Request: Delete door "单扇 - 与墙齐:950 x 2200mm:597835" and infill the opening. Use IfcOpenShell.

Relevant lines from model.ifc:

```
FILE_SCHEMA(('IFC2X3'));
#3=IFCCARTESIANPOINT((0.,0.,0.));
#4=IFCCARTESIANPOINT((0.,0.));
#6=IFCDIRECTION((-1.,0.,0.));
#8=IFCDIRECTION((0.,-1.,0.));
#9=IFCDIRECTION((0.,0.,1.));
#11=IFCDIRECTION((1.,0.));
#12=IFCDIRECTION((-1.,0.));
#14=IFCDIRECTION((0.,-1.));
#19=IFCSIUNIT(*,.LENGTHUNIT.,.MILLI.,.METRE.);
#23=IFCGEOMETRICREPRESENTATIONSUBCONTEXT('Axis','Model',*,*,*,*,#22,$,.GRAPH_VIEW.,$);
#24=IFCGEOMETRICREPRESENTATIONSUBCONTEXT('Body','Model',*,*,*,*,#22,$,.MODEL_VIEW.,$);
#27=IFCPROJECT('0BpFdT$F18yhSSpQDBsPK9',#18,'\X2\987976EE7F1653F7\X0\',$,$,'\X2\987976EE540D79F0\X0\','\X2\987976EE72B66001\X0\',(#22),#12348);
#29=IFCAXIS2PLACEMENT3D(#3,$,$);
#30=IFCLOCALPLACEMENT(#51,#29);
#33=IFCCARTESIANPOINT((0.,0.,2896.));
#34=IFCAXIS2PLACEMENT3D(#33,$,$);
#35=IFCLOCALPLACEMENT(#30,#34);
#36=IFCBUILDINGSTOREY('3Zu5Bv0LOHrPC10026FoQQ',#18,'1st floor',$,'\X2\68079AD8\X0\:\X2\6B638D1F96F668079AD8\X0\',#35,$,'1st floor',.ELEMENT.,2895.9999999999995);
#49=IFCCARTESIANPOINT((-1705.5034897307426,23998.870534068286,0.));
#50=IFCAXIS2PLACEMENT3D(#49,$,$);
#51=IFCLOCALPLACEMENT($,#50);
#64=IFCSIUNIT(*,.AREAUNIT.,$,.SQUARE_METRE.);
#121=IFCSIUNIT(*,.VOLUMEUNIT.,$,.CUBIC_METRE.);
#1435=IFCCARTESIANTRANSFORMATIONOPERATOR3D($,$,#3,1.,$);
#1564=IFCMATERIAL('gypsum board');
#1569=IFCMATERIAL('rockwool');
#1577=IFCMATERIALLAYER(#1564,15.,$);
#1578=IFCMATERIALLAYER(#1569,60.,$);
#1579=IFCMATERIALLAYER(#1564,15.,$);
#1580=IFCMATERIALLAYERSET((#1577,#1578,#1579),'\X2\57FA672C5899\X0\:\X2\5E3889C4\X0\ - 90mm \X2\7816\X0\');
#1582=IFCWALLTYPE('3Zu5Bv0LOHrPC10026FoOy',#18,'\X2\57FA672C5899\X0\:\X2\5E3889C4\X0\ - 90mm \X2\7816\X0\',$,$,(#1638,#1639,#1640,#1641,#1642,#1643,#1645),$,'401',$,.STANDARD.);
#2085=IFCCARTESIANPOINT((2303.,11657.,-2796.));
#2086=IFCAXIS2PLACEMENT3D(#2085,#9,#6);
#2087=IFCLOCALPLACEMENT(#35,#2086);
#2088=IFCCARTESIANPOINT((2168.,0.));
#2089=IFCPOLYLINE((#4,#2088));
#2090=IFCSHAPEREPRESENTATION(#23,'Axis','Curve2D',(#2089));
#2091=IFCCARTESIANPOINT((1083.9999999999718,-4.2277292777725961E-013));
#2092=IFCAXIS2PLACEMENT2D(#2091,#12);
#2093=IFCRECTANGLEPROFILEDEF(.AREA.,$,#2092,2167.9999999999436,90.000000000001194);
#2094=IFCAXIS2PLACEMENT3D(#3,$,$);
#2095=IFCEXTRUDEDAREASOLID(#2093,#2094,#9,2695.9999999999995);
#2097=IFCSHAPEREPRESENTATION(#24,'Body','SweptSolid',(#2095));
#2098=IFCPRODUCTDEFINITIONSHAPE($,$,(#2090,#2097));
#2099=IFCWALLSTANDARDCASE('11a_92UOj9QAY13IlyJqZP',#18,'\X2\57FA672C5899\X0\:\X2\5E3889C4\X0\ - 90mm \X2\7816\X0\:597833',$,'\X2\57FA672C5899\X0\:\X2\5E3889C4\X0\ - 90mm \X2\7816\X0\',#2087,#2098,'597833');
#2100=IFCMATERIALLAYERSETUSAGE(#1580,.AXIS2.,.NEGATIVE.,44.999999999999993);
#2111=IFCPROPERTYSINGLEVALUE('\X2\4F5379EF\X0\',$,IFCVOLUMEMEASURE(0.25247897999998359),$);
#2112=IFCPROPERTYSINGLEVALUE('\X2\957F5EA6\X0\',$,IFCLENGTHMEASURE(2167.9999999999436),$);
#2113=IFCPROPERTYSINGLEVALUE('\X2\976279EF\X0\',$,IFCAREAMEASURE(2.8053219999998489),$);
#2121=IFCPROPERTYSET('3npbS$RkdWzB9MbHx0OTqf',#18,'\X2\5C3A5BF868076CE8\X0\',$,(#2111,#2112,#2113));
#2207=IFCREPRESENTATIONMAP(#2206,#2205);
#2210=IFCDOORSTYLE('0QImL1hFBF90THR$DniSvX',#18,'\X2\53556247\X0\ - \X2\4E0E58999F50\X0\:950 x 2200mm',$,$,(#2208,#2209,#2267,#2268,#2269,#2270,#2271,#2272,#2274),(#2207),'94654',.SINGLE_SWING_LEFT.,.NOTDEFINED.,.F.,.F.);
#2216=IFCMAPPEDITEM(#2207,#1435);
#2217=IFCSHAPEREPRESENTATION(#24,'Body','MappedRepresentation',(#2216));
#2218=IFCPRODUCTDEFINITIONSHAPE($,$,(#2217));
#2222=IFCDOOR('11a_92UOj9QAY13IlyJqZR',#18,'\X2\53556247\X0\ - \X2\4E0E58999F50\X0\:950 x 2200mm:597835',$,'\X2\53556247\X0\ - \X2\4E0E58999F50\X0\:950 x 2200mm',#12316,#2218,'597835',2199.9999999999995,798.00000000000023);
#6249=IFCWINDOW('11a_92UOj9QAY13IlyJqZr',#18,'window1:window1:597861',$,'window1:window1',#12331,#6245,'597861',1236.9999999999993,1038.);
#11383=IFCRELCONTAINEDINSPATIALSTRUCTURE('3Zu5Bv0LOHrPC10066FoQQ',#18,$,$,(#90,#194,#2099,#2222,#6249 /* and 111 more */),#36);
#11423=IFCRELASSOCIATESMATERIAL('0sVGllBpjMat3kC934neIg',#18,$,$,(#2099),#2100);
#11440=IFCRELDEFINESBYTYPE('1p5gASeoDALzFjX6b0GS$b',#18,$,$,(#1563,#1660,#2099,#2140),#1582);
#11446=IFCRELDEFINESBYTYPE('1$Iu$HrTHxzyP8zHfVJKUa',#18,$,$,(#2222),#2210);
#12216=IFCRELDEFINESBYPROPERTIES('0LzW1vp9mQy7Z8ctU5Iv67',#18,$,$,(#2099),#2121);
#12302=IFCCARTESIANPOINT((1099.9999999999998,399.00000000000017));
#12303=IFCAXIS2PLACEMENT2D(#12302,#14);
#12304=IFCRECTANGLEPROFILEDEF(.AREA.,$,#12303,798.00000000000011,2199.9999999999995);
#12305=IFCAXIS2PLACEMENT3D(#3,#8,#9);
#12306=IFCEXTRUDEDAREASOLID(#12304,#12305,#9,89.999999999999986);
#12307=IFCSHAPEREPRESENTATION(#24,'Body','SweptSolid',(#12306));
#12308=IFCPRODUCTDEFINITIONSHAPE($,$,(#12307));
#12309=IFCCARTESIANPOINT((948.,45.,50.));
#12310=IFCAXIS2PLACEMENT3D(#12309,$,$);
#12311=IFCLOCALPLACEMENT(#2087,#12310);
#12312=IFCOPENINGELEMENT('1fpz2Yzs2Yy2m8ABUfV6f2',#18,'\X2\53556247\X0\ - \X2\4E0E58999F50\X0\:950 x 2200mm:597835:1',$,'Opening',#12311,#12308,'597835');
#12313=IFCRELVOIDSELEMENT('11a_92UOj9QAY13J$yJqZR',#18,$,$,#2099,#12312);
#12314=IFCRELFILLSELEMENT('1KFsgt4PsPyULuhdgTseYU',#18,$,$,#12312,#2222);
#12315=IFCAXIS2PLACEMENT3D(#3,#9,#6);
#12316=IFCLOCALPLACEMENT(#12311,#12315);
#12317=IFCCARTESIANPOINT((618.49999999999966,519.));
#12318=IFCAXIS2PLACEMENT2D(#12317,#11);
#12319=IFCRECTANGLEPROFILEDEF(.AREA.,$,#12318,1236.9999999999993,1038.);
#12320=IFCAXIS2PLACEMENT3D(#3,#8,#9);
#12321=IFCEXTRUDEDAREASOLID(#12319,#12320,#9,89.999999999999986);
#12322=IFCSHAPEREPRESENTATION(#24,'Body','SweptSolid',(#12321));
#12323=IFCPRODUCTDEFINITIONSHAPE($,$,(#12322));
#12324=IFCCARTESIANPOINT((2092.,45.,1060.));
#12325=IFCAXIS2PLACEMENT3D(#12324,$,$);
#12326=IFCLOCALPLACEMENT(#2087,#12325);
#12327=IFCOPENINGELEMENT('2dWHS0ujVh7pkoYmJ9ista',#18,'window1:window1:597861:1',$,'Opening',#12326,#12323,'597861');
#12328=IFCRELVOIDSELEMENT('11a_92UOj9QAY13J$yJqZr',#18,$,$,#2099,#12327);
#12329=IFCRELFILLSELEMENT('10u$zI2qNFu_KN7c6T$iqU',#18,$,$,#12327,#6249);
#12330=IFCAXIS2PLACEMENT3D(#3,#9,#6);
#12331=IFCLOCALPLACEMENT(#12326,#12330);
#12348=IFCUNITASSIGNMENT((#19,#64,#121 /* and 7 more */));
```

```python
import ifcopenshell
import ifcopenshell.api.feature
import ifcopenshell.api.pset
import ifcopenshell.api.root
import ifcopenshell.geom
import ifcopenshell.util.element
import ifcopenshell.util.shape
import ifcopenshell.util.unit

model = ifcopenshell.open("model.ifc")
area_scale = ifcopenshell.util.unit.calculate_unit_scale(model, "AREAUNIT")
volume_scale = ifcopenshell.util.unit.calculate_unit_scale(model, "VOLUMEUNIT")
settings = ifcopenshell.geom.settings()


def volume(element):
    """Net volume in cubic metres, openings subtracted."""
    shape = ifcopenshell.geom.create_shape(settings, element)
    return ifcopenshell.util.shape.get_volume(shape.geometry)


door = model.by_guid("11a_92UOj9QAY13IlyJqZR")
opening = door.FillsVoids[0].RelatingOpeningElement
wall = opening.VoidsElements[0].RelatingBuildingElement
before = volume(wall)

ifcopenshell.api.root.remove_product(model, product=door)
ifcopenshell.api.feature.remove_feature(model, feature=opening)

after = volume(wall)
thickness = 0.09  # wall thickness in metres

# Update the wall's stored quantities.
pset = model.by_id(ifcopenshell.util.element.get_pset(wall, "尺寸标注", should_inherit=False)["id"])
ifcopenshell.api.pset.edit_pset(model, pset=pset, properties={
    "体积": model.create_entity("IfcVolumeMeasure", after / volume_scale),
    "面积": model.create_entity("IfcAreaMeasure", after / thickness / area_scale),
})

print(f"wall volume {before:.3f} -> {after:.3f} m3")

model.write("model_v2.ifc")
```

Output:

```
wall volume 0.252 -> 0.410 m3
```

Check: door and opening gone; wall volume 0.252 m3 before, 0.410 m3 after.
